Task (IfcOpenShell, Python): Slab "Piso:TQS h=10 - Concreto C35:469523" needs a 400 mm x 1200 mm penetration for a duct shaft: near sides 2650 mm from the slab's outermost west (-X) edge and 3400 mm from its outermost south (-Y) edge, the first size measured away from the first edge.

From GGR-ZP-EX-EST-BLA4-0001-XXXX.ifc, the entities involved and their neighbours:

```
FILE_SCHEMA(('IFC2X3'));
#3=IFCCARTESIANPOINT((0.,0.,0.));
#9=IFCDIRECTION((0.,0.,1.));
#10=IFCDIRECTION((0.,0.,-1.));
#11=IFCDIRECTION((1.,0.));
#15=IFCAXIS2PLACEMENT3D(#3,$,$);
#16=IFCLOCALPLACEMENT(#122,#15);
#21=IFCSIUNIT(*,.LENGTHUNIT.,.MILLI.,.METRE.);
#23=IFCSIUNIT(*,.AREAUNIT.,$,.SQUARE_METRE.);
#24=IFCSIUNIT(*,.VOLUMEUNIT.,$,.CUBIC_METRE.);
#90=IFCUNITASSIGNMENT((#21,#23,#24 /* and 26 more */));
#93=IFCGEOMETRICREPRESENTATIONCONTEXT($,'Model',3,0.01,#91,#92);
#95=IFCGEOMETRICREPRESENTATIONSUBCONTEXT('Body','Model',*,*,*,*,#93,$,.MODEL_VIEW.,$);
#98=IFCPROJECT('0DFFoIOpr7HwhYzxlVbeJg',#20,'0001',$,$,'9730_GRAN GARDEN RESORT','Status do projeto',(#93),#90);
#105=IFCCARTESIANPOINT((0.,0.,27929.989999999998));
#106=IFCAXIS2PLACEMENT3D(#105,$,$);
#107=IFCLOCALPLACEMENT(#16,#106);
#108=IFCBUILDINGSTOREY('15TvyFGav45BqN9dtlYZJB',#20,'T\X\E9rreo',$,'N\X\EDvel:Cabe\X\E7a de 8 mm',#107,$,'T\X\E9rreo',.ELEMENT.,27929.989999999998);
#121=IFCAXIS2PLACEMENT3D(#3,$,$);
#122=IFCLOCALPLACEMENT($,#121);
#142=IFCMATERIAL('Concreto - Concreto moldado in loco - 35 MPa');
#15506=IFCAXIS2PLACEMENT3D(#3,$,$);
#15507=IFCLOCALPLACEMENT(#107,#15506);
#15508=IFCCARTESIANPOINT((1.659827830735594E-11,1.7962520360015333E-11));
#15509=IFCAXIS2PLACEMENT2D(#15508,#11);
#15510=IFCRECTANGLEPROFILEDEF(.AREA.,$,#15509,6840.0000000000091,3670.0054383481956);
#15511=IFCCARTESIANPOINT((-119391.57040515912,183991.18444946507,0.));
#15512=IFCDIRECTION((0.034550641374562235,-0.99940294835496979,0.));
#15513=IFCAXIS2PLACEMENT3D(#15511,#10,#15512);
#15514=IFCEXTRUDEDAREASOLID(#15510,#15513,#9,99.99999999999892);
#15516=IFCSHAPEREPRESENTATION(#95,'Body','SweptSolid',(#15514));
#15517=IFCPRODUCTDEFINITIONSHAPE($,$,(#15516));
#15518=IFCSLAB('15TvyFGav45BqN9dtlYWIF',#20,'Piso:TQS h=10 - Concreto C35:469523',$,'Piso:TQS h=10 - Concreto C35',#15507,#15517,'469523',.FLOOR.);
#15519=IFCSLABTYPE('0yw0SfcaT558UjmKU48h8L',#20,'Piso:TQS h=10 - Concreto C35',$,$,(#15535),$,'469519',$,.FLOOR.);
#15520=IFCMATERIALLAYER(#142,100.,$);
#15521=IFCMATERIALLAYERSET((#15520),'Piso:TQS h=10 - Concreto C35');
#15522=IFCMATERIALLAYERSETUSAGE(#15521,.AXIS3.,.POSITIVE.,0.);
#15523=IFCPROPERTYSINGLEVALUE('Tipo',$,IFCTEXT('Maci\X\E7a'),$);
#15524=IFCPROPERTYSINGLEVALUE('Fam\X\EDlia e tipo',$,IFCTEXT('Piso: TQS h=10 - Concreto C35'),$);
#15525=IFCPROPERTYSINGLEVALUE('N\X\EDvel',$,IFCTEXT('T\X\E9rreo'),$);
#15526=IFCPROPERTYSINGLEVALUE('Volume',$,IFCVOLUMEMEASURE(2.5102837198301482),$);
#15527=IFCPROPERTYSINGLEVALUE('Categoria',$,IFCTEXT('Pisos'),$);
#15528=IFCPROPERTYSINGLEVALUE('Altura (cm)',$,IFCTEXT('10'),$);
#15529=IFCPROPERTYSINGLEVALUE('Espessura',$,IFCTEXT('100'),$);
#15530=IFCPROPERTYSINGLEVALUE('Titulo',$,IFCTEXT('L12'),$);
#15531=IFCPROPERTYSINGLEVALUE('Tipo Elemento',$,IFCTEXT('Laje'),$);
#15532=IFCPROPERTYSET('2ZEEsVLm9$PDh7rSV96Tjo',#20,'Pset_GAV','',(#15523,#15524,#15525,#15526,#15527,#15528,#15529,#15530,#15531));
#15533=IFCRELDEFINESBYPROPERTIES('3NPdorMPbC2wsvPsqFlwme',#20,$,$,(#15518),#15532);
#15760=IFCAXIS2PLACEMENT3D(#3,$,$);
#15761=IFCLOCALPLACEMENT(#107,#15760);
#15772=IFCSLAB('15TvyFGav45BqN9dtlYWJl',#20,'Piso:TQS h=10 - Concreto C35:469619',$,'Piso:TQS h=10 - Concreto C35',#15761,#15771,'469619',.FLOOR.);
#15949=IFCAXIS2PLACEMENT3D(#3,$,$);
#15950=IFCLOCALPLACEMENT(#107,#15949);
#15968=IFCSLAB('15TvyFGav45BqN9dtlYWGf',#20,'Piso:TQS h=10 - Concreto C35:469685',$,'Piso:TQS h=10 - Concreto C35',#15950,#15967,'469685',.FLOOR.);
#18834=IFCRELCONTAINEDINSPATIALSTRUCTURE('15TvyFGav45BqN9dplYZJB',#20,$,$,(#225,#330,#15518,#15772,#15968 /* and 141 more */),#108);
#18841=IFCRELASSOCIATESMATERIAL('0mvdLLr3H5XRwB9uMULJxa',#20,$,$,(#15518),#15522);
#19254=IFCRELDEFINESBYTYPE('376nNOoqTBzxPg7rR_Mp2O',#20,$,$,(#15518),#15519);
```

```python
import numpy as np
import ifcopenshell
import ifcopenshell.api.feature
import ifcopenshell.api.geometry
import ifcopenshell.api.pset
import ifcopenshell.api.root
import ifcopenshell.geom
import ifcopenshell.util.element
import ifcopenshell.util.placement
import ifcopenshell.util.representation
import ifcopenshell.util.shape
import ifcopenshell.util.unit

model = ifcopenshell.open("GGR-ZP-EX-EST-BLA4-0001-XXXX.ifc")
unit_scale = ifcopenshell.util.unit.calculate_unit_scale(model)
volume_scale = ifcopenshell.util.unit.calculate_unit_scale(model, "VOLUMEUNIT")
settings = ifcopenshell.geom.settings()


def volume(element):
    """Net volume in cubic metres, openings subtracted."""
    shape = ifcopenshell.geom.create_shape(settings, element)
    return ifcopenshell.util.shape.get_volume(shape.geometry)


slab = model.by_guid("15TvyFGav45BqN9dtlYWIF")
before = volume(slab)

# Extent in the slab's own axes, in metres. The edges named are its -X and -Y sides.
slab_shape = ifcopenshell.geom.create_shape(settings, slab)
vertices = ifcopenshell.util.shape.get_vertices(slab_shape.geometry)
x_min, y_min, bottom = vertices.min(axis=0)
top = vertices[:, 2].max()

opening = ifcopenshell.api.root.create_entity(model, ifc_class="IfcOpeningElement", name="Duct shaft opening")
context = ifcopenshell.util.representation.get_context(model, "Model", "Body", "MODEL_VIEW")
width, depth = 0.4, 1.2
outline = [(0.0, 0.0), (width, 0.0), (width, depth), (0.0, depth), (0.0, 0.0)]
# Overshoot both faces by 50 mm so the cut is clean.
shape = ifcopenshell.api.geometry.add_slab_representation(
    model, context=context, depth=top - bottom + 0.1, polyline=outline
)
ifcopenshell.api.geometry.assign_representation(model, product=opening, representation=shape)

matrix = ifcopenshell.util.placement.get_local_placement(slab.ObjectPlacement)
matrix[:, 3] = matrix @ np.append(np.array([x_min + 2.65, y_min + 3.4, bottom - 0.05]) / unit_scale, 1.0)
ifcopenshell.api.geometry.edit_object_placement(model, product=opening, matrix=matrix, is_si=False)
ifcopenshell.api.feature.add_feature(model, feature=opening, element=slab)

after = volume(slab)

# Update the slab's stored quantities.
pset = model.by_id(ifcopenshell.util.element.get_pset(slab, "Pset_GAV", should_inherit=False)["id"])
ifcopenshell.api.pset.edit_pset(model, pset=pset, properties={
    "Volume": model.create_entity("IfcVolumeMeasure", after / volume_scale),
})

print(f"slab volume {before:.3f} -> {after:.3f} m3")

model.write("GGR-ZP-EX-EST-BLA4-0001-XXXX_v2.ifc")
```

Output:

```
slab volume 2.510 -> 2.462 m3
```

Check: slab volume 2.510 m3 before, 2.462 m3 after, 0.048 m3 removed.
